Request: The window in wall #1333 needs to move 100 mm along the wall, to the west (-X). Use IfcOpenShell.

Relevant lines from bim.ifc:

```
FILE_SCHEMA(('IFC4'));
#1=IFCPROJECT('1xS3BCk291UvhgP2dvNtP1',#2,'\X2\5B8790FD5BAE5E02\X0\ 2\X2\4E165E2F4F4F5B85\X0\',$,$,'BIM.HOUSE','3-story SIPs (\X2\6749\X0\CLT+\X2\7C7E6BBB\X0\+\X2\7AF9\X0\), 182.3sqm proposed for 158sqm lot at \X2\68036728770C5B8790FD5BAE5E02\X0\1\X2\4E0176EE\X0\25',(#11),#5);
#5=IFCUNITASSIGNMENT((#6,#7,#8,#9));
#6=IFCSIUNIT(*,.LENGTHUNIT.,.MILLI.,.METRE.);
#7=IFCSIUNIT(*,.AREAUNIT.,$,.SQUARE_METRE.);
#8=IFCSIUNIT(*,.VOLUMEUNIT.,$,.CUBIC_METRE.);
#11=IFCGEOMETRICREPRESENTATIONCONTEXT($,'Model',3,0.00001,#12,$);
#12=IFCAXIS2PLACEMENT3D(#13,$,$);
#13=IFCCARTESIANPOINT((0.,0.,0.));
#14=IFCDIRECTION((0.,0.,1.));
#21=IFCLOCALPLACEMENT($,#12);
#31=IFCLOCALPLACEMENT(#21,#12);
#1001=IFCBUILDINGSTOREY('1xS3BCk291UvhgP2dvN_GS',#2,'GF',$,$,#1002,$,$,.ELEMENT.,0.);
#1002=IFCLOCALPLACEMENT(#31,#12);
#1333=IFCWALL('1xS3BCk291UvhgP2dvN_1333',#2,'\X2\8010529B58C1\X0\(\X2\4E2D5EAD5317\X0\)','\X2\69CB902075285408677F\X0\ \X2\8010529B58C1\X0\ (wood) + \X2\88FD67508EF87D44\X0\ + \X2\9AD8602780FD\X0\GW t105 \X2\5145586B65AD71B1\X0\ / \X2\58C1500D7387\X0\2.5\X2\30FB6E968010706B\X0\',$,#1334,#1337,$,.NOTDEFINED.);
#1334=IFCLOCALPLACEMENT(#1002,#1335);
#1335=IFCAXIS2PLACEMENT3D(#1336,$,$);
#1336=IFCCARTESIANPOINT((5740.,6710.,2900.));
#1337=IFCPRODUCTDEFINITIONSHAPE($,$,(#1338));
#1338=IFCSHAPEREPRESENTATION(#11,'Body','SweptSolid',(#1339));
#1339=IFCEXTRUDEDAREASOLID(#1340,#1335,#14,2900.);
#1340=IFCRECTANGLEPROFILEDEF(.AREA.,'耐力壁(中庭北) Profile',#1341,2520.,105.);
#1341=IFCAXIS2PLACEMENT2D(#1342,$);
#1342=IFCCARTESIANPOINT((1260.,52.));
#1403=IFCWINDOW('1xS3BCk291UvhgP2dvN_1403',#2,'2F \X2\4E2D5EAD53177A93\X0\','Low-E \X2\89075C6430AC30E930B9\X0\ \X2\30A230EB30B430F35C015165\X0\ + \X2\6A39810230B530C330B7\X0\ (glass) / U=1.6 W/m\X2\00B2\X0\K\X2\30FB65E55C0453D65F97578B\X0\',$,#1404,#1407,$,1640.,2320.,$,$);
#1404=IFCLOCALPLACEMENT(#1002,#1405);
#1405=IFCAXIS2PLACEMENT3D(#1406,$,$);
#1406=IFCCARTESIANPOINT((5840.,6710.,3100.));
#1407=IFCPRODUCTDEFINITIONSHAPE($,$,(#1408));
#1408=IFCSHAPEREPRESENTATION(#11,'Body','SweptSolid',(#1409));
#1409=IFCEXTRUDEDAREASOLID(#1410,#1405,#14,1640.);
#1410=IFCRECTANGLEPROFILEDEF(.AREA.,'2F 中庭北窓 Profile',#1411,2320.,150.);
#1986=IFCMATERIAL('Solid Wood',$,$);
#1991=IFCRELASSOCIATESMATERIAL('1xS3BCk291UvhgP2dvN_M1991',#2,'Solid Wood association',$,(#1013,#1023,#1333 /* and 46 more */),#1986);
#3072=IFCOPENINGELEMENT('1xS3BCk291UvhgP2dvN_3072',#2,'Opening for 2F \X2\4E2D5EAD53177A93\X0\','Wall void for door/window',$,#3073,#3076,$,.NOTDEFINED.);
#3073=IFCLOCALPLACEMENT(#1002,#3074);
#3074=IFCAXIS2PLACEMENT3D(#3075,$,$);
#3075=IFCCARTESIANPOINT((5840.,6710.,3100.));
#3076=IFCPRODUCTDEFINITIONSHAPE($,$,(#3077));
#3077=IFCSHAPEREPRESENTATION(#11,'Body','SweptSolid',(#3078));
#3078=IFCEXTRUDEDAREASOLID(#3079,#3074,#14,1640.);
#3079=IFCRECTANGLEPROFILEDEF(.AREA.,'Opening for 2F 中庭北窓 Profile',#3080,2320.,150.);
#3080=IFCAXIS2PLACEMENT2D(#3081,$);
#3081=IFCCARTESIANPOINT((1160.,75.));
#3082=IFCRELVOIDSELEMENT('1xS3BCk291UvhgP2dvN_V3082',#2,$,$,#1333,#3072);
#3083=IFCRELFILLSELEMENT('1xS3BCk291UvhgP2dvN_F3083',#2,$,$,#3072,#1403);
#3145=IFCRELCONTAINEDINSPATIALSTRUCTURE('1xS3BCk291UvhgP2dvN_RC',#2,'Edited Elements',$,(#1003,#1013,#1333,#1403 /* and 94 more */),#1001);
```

```python
import ifcopenshell
import ifcopenshell.api.geometry
import ifcopenshell.util.placement

model = ifcopenshell.open("bim.ifc")

window = model.by_guid("1xS3BCk291UvhgP2dvN_1403")
opening = window.FillsVoids[0].RelatingOpeningElement
wall = opening.VoidsElements[0].RelatingBuildingElement

wall_matrix = ifcopenshell.util.placement.get_local_placement(wall.ObjectPlacement)
shift = wall_matrix[:3, 0] * -100.0
before = ifcopenshell.util.placement.get_local_placement(window.ObjectPlacement)[:3, 3].copy()

# The window is not placed relative to its opening, so move both.
for product in (opening, window):
    matrix = ifcopenshell.util.placement.get_local_placement(product.ObjectPlacement)
    matrix[:3, 3] += shift
    ifcopenshell.api.geometry.edit_object_placement(model, product=product, matrix=matrix, is_si=False)

after = ifcopenshell.util.placement.get_local_placement(window.ObjectPlacement)[:3, 3]
print("window moved by", (after - before).round(3) + 0.0)

model.write("bim_edited.ifc")
```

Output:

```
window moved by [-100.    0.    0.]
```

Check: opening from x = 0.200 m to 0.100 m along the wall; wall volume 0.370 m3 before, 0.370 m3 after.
